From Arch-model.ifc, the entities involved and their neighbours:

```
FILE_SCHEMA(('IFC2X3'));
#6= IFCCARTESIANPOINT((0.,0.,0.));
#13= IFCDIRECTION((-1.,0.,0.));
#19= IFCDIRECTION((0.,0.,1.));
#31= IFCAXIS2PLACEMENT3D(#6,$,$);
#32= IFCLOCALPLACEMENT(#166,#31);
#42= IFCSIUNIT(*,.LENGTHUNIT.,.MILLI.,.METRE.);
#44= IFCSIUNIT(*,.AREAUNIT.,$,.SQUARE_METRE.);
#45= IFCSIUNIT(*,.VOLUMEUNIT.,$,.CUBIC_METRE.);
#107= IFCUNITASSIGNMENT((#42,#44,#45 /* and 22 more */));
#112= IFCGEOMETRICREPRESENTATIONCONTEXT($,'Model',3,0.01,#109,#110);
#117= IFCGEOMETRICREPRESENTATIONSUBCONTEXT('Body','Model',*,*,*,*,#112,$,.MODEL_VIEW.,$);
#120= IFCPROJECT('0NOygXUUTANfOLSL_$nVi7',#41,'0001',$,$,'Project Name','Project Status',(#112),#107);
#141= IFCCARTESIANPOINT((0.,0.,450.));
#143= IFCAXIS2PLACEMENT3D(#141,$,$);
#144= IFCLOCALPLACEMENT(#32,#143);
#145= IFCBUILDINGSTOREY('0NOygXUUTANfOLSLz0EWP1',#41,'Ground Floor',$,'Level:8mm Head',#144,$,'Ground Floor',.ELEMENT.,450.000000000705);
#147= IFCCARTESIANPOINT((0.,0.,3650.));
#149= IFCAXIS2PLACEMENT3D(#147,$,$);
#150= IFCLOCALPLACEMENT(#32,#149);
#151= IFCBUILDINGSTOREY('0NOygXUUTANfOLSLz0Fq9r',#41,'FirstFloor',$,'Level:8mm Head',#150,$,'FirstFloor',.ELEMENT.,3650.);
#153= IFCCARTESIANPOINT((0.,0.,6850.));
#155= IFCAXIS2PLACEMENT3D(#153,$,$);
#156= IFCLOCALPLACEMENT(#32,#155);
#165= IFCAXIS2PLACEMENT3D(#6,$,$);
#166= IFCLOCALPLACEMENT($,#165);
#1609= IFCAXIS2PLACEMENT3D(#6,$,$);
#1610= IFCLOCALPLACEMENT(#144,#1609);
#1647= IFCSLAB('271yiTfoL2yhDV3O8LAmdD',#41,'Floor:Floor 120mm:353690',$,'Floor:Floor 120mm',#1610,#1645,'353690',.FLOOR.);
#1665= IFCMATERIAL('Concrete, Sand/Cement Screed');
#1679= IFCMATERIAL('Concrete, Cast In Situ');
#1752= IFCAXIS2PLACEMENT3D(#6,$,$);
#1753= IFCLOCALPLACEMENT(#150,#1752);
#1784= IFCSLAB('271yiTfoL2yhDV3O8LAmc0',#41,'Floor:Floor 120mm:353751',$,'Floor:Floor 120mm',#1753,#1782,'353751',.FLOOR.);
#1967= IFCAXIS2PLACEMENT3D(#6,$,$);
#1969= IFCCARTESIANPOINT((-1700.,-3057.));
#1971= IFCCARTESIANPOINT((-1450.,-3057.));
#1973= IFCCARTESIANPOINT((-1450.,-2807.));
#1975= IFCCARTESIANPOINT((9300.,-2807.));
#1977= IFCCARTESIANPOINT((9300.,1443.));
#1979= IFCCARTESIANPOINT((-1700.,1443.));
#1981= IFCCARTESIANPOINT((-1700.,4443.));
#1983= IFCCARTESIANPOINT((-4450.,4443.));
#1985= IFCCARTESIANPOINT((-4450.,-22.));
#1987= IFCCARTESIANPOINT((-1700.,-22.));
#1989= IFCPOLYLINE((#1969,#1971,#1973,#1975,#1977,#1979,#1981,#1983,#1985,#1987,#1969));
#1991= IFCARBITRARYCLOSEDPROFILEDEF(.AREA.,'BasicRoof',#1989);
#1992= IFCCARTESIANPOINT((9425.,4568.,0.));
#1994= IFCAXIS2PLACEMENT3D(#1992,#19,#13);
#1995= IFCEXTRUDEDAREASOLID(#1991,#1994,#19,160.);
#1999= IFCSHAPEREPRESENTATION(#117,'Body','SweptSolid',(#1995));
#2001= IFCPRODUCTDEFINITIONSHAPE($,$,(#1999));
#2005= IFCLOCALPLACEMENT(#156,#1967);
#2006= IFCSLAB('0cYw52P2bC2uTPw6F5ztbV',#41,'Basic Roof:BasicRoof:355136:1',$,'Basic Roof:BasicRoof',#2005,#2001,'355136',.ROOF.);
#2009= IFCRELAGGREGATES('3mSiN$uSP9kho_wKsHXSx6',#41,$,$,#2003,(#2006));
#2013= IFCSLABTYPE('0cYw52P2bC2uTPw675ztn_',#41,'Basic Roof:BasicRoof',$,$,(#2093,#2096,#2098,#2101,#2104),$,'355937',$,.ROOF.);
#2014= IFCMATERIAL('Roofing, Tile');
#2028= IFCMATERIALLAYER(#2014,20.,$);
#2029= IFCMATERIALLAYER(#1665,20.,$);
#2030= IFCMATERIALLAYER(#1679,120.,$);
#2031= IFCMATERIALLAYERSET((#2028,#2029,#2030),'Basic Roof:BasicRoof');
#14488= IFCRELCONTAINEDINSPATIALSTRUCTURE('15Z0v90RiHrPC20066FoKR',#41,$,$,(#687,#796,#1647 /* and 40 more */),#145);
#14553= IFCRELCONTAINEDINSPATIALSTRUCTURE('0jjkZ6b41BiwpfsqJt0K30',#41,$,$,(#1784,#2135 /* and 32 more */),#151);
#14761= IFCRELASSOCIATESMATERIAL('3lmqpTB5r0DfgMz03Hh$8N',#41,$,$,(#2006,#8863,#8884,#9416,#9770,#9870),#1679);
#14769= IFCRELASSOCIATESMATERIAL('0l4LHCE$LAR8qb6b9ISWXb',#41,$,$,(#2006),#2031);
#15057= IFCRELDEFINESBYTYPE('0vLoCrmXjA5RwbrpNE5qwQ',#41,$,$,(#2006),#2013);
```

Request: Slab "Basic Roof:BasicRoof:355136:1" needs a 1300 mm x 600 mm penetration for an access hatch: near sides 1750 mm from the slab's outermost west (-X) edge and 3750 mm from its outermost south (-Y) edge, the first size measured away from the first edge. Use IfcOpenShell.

```python
import numpy as np
import ifcopenshell
import ifcopenshell.api.feature
import ifcopenshell.api.geometry
import ifcopenshell.api.root
import ifcopenshell.geom
import ifcopenshell.util.placement
import ifcopenshell.util.representation
import ifcopenshell.util.shape
import ifcopenshell.util.unit

model = ifcopenshell.open("Arch-model.ifc")
unit_scale = ifcopenshell.util.unit.calculate_unit_scale(model)
settings = ifcopenshell.geom.settings()


def volume(element):
    """Net volume in cubic metres, openings subtracted."""
    shape = ifcopenshell.geom.create_shape(settings, element)
    return ifcopenshell.util.shape.get_volume(shape.geometry)


slab = model.by_guid("0cYw52P2bC2uTPw6F5ztbV")
before = volume(slab)

# Extent in the slab's own axes, in metres. The edges named are its -X and -Y sides.
slab_shape = ifcopenshell.geom.create_shape(settings, slab)
vertices = ifcopenshell.util.shape.get_vertices(slab_shape.geometry)
x_min, y_min, bottom = vertices.min(axis=0)
top = vertices[:, 2].max()

opening = ifcopenshell.api.root.create_entity(model, ifc_class="IfcOpeningElement", name="Access hatch opening")
context = ifcopenshell.util.representation.get_context(model, "Model", "Body", "MODEL_VIEW")
width, depth = 1.3, 0.6
outline = [(0.0, 0.0), (width, 0.0), (width, depth), (0.0, depth), (0.0, 0.0)]
# Overshoot both faces by 50 mm so the cut is clean.
shape = ifcopenshell.api.geometry.add_slab_representation(
    model, context=context, depth=top - bottom + 0.1, polyline=outline
)
ifcopenshell.api.geometry.assign_representation(model, product=opening, representation=shape)

matrix = ifcopenshell.util.placement.get_local_placement(slab.ObjectPlacement)
matrix[:, 3] = matrix @ np.append(np.array([x_min + 1.75, y_min + 3.75, bottom - 0.05]) / unit_scale, 1.0)
ifcopenshell.api.geometry.edit_object_placement(model, product=opening, matrix=matrix, is_si=False)
ifcopenshell.api.feature.add_feature(model, feature=opening, element=slab)

after = volume(slab)

print(f"slab volume {before:.3f} -> {after:.3f} m3")

model.write("Arch-model_rev.ifc")
```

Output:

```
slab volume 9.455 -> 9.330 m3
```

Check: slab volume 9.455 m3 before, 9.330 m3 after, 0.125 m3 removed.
